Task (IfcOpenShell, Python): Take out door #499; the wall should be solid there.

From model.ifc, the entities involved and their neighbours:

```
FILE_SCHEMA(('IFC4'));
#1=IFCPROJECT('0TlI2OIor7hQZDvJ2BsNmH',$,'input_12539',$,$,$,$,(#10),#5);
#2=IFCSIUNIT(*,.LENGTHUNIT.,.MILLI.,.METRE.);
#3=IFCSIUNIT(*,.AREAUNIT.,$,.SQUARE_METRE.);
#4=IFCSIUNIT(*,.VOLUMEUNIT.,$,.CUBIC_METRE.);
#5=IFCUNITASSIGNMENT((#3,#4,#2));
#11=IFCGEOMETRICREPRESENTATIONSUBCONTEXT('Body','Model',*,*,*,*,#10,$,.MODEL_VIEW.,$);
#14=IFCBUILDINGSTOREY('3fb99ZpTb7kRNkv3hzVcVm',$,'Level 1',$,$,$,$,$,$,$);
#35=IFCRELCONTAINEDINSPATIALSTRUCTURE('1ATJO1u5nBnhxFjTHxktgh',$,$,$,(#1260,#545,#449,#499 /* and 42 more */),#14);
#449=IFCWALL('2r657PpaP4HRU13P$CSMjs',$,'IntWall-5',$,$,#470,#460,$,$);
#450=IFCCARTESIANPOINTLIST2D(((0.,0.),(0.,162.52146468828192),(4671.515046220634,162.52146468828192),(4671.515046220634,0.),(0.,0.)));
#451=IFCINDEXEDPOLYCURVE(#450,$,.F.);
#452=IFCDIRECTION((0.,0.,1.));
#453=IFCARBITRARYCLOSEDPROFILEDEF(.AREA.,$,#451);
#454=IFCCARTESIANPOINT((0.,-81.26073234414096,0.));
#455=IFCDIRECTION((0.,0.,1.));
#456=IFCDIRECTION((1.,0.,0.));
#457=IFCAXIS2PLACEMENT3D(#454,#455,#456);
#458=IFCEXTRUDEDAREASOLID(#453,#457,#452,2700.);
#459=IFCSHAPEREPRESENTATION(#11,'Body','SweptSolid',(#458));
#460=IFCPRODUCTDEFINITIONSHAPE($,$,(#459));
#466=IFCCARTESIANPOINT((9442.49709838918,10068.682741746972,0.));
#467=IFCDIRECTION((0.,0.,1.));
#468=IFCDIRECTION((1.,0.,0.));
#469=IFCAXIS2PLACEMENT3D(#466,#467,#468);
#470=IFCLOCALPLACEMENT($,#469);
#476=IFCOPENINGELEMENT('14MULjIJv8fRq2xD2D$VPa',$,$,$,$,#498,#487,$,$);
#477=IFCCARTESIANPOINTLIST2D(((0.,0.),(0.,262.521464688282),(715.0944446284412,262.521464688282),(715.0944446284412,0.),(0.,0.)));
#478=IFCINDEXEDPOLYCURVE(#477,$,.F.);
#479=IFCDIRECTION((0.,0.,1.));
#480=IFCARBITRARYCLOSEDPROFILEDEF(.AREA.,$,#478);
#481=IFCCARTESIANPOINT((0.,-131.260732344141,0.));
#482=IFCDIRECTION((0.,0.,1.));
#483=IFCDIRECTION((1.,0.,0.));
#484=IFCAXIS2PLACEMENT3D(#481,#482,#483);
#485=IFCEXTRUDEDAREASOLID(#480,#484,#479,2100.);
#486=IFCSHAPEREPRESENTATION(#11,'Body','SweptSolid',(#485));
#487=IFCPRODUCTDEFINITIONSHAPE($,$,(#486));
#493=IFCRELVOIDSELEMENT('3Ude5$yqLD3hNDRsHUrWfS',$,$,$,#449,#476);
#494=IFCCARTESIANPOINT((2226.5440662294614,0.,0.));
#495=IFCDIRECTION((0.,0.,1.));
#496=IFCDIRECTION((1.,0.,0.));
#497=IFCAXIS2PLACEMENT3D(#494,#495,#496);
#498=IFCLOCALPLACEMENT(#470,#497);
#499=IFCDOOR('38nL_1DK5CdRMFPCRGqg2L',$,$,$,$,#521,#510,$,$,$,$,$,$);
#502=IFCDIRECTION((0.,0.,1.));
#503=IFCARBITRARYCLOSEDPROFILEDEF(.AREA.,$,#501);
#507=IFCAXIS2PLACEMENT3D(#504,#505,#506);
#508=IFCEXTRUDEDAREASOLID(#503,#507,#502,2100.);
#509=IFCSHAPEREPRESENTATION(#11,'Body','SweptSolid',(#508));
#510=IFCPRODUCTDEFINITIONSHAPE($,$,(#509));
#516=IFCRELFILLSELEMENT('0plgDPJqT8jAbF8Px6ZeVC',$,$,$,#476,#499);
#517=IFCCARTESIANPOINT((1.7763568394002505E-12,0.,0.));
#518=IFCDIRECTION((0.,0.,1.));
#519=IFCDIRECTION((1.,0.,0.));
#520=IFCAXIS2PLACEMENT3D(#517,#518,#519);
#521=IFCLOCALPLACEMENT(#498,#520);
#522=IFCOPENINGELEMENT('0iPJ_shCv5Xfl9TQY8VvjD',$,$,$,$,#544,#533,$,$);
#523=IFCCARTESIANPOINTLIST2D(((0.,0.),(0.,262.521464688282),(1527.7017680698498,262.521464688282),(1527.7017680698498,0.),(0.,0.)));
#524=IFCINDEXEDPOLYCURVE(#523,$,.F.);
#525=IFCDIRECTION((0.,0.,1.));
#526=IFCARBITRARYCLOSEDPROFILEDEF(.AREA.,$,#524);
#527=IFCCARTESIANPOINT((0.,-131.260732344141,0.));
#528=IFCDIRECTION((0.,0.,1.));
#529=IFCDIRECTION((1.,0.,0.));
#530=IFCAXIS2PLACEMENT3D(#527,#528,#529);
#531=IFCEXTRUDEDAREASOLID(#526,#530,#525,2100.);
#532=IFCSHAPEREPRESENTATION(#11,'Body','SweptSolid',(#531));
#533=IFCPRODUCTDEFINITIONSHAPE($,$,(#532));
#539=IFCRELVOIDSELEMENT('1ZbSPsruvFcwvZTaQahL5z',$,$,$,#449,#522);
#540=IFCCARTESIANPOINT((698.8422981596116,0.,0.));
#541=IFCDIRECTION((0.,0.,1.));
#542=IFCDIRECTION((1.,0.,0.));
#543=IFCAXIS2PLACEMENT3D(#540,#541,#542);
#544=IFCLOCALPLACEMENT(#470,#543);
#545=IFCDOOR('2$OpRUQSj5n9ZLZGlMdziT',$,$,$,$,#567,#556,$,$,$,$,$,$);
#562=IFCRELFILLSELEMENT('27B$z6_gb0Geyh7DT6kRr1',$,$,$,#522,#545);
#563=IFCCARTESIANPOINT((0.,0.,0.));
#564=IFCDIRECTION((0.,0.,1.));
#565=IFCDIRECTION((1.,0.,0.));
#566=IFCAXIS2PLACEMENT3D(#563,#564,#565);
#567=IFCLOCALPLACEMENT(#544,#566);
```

```python
import ifcopenshell
import ifcopenshell.api.feature
import ifcopenshell.api.root
import ifcopenshell.geom
import ifcopenshell.util.shape

model = ifcopenshell.open("model.ifc")
settings = ifcopenshell.geom.settings()


def volume(element):
    """Net volume in cubic metres, openings subtracted."""
    shape = ifcopenshell.geom.create_shape(settings, element)
    return ifcopenshell.util.shape.get_volume(shape.geometry)


door = model.by_guid("38nL_1DK5CdRMFPCRGqg2L")
opening = door.FillsVoids[0].RelatingOpeningElement
wall = opening.VoidsElements[0].RelatingBuildingElement
before = volume(wall)

ifcopenshell.api.root.remove_product(model, product=door)
ifcopenshell.api.feature.remove_feature(model, feature=opening)

after = volume(wall)

print(f"wall volume {before:.3f} -> {after:.3f} m3")

model.write("model-out.ifc")
```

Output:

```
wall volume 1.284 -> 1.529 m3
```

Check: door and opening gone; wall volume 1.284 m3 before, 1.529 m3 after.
